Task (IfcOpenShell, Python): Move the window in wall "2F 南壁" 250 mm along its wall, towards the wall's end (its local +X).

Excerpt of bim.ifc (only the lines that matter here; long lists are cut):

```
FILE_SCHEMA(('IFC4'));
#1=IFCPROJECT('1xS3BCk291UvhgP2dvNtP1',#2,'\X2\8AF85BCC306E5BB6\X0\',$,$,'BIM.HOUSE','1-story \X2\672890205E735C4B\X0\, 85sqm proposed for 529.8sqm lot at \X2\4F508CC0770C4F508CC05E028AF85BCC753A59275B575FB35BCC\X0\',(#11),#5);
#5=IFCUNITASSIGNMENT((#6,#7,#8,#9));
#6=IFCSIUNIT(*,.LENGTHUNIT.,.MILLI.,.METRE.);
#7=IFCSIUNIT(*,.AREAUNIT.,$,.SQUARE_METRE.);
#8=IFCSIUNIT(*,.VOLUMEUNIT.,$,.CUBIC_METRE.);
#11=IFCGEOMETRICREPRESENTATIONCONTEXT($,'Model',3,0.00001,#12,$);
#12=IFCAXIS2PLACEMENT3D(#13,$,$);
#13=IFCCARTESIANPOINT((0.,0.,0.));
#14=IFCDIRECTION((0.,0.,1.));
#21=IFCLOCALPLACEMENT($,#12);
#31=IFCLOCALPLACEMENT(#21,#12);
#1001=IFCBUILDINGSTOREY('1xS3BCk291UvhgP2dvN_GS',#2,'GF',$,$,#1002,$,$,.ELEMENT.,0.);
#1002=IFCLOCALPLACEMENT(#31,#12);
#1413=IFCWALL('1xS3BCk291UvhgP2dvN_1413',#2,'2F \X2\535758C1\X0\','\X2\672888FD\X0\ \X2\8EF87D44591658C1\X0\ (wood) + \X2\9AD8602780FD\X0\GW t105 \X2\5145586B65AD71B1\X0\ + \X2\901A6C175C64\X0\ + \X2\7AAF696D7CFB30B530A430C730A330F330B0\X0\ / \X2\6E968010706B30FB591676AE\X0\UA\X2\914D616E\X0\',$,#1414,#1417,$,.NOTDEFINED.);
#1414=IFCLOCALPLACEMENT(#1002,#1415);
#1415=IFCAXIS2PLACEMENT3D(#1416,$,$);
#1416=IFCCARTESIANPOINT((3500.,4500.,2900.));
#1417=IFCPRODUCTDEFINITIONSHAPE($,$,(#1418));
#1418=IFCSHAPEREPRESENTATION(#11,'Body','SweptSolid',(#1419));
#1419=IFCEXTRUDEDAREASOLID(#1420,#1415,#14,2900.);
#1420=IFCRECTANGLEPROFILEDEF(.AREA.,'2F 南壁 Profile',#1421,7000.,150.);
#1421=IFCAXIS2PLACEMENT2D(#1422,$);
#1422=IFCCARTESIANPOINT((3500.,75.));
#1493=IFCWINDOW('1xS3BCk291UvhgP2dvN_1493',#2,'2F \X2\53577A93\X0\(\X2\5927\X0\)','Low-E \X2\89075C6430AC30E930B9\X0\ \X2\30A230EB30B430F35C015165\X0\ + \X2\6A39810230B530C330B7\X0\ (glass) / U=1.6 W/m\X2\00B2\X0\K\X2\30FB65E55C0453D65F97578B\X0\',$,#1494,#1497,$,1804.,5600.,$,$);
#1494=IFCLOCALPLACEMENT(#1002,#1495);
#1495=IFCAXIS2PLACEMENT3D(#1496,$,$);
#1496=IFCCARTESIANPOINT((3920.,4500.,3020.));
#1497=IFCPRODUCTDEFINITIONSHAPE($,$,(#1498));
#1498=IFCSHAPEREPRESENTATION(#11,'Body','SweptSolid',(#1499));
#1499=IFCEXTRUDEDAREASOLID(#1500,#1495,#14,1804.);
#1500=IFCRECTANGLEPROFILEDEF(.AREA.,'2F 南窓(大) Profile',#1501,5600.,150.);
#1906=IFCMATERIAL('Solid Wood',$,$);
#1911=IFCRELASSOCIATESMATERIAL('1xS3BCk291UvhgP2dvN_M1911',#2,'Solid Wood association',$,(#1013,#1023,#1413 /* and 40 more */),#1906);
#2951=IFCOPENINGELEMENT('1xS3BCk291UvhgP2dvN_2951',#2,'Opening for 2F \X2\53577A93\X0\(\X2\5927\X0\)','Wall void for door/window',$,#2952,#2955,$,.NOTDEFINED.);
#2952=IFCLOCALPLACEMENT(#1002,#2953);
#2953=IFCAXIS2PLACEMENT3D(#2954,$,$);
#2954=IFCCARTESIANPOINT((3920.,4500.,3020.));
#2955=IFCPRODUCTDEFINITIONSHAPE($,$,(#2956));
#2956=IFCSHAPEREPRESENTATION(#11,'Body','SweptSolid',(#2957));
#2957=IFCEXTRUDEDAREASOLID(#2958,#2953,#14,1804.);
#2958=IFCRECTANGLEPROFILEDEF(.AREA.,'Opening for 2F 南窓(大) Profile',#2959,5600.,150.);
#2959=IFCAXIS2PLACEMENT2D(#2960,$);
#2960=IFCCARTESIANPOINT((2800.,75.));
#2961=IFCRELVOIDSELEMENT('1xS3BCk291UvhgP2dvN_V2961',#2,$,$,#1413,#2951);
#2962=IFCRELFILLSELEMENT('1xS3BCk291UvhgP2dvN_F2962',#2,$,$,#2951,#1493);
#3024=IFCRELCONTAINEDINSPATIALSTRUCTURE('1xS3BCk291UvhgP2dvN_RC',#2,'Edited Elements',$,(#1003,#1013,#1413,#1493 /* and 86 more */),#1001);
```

```python
import ifcopenshell
import ifcopenshell.api.geometry
import ifcopenshell.util.placement
import ifcopenshell.util.unit

model = ifcopenshell.open("bim.ifc")
unit_scale = ifcopenshell.util.unit.calculate_unit_scale(model)

window = model.by_guid("1xS3BCk291UvhgP2dvN_1493")
opening = window.FillsVoids[0].RelatingOpeningElement
wall = opening.VoidsElements[0].RelatingBuildingElement

wall_matrix = ifcopenshell.util.placement.get_local_placement(wall.ObjectPlacement)
shift = wall_matrix[:3, 0] * 0.25 / unit_scale
before = ifcopenshell.util.placement.get_local_placement(window.ObjectPlacement)[:3, 3].copy()

# The window is not placed relative to its opening, so move both.
for product in (opening, window):
    matrix = ifcopenshell.util.placement.get_local_placement(product.ObjectPlacement)
    matrix[:3, 3] += shift
    ifcopenshell.api.geometry.edit_object_placement(model, product=product, matrix=matrix, is_si=False)

after = ifcopenshell.util.placement.get_local_placement(window.ObjectPlacement)[:3, 3]
print("window moved by", (after - before).round(3) + 0.0)

model.write("bim-out.ifc")
```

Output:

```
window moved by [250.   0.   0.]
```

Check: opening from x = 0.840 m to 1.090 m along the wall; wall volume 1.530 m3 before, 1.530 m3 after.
